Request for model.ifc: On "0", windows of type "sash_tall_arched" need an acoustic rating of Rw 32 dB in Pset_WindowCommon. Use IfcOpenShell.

First a look at what the model holds.

```python
import ifcopenshell
import ifcopenshell.util.element

model = ifcopenshell.open("model.ifc")
print(model.schema)
storey = next(s for s in model.by_type("IfcBuildingStorey") if s.Name == "0")
windows = [e for e in ifcopenshell.util.element.get_decomposition(storey) if e.is_a("IfcWindow")]
seen = {}
for e in windows:
    element_type = ifcopenshell.util.element.get_type(e)
    key = (element_type.Name if element_type != e and element_type else None, ifcopenshell.util.element.get_pset(e, "Pset_WindowCommon", "AcousticRating"))
    seen[key] = seen.get(key, 0) + 1
for (name, value), count in sorted(seen.items(), key=str):
    print(count, "x", name, "|", value)
```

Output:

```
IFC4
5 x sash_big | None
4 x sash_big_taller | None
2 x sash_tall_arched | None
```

```python
import ifcopenshell
import ifcopenshell.api.pset
import ifcopenshell.util.element

model = ifcopenshell.open("model.ifc")

storey = next(s for s in model.by_type("IfcBuildingStorey") if s.Name == "0")
windows = [e for e in ifcopenshell.util.element.get_decomposition(storey) if e.is_a("IfcWindow")]

count = 0
for e in windows:
    element_type = ifcopenshell.util.element.get_type(e)
    if element_type in (None, e) or element_type.Name != "sash_tall_arched":
        continue
    # add_pset returns the element's existing set when there is one.
    pset = ifcopenshell.api.pset.add_pset(model, product=e, name="Pset_WindowCommon")
    ifcopenshell.api.pset.edit_pset(model, pset=pset, properties={"AcousticRating": "Rw 32 dB"})
    count += 1

print(count, "windows updated")

model.write("model_updated.ifc")
```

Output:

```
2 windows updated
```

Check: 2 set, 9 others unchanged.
